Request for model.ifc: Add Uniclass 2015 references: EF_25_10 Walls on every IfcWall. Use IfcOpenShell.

First a look at what the model holds.

```python
import ifcopenshell

model = ifcopenshell.open("model.ifc")
print(model.schema)
print("classifications:", [c.Name for c in model.by_type("IfcClassification")])
for ifc_class in ("IfcDoor", "IfcRoof", "IfcStair", "IfcWall", "IfcWindow"):
    print(ifc_class, len(model.by_type(ifc_class)))
```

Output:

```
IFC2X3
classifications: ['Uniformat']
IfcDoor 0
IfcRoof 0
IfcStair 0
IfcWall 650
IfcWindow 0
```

```python
import ifcopenshell
import ifcopenshell.api.classification

model = ifcopenshell.open("model.ifc")

# IFC2X3 requires Source and Edition and has no link from the project to the system.
system = model.create_entity("IfcClassification", Source="NBS", Edition="2015", Name="Uniclass 2015")

codes = {
    "IfcWall": ("EF_25_10", "Walls"),
}
for ifc_class, (code, name) in codes.items():
    products = model.by_type(ifc_class)
    ifcopenshell.api.classification.add_reference(
        model, products=products, classification=system, identification=code, name=name
    )
    print(code, len(products))

model.write("model-out.ifc")
```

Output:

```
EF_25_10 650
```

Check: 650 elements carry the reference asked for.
